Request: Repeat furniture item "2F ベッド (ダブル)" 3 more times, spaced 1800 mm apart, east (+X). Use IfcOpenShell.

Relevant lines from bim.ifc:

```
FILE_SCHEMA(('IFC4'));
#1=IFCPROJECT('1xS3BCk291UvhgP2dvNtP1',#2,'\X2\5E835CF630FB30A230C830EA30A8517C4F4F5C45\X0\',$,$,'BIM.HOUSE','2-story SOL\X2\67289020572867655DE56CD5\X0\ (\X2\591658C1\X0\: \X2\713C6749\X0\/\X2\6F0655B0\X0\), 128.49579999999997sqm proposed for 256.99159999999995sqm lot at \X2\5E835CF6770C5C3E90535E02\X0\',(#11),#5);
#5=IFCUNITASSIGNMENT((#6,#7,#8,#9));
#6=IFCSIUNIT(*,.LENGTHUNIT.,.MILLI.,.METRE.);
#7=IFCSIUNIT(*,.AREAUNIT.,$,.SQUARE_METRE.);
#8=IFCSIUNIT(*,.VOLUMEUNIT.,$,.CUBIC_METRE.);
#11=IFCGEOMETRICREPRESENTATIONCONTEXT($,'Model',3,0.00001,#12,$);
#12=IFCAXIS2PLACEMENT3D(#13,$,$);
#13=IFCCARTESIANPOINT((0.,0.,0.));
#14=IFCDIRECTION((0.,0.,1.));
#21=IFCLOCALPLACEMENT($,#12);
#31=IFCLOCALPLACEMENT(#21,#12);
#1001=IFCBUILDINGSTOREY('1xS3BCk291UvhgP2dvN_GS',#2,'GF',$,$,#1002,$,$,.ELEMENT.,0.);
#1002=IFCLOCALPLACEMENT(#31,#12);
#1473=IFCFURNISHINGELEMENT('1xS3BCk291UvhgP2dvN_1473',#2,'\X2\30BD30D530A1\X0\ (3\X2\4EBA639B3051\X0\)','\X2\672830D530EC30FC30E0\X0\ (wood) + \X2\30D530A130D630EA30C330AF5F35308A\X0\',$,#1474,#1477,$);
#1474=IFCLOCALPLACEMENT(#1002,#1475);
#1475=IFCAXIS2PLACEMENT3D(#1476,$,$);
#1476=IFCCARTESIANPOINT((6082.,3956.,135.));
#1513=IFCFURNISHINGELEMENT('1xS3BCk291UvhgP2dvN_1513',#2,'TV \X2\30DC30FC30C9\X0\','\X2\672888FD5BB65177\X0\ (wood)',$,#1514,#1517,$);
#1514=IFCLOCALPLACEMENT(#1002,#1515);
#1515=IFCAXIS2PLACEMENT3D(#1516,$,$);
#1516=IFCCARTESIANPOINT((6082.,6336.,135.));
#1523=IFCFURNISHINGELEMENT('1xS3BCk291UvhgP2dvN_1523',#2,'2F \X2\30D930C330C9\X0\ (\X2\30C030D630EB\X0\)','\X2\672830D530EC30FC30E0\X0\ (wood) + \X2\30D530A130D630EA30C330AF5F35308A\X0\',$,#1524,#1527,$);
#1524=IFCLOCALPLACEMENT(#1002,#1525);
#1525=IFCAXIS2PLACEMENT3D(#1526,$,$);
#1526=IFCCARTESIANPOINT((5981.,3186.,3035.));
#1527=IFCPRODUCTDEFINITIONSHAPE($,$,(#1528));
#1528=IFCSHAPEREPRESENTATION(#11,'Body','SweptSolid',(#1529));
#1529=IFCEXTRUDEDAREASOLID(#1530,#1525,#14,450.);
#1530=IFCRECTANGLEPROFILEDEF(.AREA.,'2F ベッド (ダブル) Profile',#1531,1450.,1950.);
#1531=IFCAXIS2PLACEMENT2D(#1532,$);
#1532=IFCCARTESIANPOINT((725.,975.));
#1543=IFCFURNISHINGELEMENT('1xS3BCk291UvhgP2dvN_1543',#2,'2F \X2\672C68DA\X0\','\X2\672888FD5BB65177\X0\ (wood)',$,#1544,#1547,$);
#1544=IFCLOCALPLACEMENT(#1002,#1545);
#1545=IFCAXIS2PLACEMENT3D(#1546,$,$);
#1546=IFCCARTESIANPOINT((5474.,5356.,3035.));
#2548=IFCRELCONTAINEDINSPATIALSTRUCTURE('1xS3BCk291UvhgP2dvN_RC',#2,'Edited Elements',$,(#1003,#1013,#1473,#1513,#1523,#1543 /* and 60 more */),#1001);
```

```python
import numpy as np
import ifcopenshell
import ifcopenshell.api.geometry
import ifcopenshell.api.root
import ifcopenshell.util.element
import ifcopenshell.util.placement
import ifcopenshell.util.unit

model = ifcopenshell.open("bim.ifc")
unit_scale = ifcopenshell.util.unit.calculate_unit_scale(model)


def reuse_history(source, copy):
    """copy_class also copies each property set's owner history, people and application; keep the originals."""
    for rel in copy.IsDefinedBy:
        if rel.is_a("IfcRelDefinesByProperties") and (history := rel.RelatingPropertyDefinition.OwnerHistory):
            rel.RelatingPropertyDefinition.OwnerHistory = source.OwnerHistory
            ifcopenshell.util.element.remove_deep2(model, history)


source = model.by_guid("1xS3BCk291UvhgP2dvN_1523")
base = ifcopenshell.util.placement.get_local_placement(source.ObjectPlacement)
step = np.array([1.0, 0.0, 0.0]) * 1.8 / unit_scale

for i in range(1, 4):
    copy = ifcopenshell.api.root.copy_class(model, product=source)
    copy.Representation = ifcopenshell.util.element.copy_deep(
        model, source.Representation, exclude=["IfcGeometricRepresentationContext", "IfcRepresentationMap"]
    )
    reuse_history(source, copy)
    matrix = base.copy()
    matrix[:3, 3] += i * step
    print("added at", matrix[:3, 3].round(3) + 0.0)
    ifcopenshell.api.geometry.edit_object_placement(model, product=copy, matrix=matrix, is_si=False)

model.write("bim-out.ifc")
```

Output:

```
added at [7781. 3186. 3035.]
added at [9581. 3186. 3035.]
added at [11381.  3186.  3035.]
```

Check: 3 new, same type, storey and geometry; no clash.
